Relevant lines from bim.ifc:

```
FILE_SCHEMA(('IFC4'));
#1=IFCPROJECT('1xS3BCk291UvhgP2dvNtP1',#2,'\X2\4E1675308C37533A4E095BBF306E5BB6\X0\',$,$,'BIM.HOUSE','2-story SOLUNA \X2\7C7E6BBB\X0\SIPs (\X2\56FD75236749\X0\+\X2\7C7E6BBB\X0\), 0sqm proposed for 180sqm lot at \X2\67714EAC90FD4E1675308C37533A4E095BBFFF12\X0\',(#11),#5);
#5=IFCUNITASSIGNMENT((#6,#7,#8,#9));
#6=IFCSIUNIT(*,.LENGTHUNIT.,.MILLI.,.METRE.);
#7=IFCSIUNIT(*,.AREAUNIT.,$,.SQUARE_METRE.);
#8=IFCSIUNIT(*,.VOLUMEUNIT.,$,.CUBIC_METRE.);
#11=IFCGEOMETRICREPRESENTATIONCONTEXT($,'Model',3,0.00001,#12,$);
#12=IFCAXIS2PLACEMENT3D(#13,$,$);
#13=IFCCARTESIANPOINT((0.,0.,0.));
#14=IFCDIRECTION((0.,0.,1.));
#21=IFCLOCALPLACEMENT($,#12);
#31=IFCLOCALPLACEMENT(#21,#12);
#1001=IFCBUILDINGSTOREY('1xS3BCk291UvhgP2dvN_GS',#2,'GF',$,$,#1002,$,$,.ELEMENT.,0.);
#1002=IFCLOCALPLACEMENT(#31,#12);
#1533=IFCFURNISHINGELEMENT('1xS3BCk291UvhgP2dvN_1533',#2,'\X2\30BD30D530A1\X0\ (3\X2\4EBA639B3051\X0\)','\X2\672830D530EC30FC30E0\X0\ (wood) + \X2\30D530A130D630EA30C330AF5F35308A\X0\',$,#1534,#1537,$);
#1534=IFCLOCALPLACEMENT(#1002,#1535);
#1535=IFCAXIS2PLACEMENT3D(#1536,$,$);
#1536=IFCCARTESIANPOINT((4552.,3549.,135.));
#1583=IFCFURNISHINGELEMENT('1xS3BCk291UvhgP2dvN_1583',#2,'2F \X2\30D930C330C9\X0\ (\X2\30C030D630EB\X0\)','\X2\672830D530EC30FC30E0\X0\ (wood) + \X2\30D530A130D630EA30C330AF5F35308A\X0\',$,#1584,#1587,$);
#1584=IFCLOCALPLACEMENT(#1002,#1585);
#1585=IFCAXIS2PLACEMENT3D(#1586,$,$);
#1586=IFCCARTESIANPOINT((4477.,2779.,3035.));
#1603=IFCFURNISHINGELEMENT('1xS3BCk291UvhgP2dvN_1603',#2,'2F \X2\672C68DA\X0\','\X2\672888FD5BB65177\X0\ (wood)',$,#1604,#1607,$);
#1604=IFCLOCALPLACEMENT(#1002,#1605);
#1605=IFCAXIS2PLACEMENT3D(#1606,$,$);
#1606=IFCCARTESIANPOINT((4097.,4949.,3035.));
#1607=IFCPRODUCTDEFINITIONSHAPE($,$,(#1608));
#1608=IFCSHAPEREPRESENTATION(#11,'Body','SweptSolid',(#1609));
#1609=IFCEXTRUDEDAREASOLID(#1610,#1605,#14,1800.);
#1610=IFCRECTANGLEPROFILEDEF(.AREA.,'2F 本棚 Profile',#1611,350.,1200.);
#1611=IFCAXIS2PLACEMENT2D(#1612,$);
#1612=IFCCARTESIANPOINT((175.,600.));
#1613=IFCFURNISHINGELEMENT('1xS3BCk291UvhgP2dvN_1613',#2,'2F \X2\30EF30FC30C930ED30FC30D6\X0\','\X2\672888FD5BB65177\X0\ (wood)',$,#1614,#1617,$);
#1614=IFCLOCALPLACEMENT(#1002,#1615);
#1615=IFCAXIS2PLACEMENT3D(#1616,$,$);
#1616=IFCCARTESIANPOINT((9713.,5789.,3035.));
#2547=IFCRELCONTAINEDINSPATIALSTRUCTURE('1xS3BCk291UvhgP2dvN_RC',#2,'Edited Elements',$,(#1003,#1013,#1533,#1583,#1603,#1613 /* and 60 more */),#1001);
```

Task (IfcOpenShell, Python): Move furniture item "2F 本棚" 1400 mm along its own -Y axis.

```python
import ifcopenshell
import ifcopenshell.api.geometry
import ifcopenshell.util.placement
import ifcopenshell.util.unit

model = ifcopenshell.open("bim.ifc")
unit_scale = ifcopenshell.util.unit.calculate_unit_scale(model)

item = model.by_guid("1xS3BCk291UvhgP2dvN_1603")
matrix = ifcopenshell.util.placement.get_local_placement(item.ObjectPlacement)
matrix[:3, 3] -= matrix[:3, 1] * 1.4 / unit_scale
ifcopenshell.api.geometry.edit_object_placement(model, product=item, matrix=matrix, is_si=False)

print(ifcopenshell.util.placement.get_local_placement(item.ObjectPlacement).round(3) + 0.0)

model.write("bim_v2.ifc")
```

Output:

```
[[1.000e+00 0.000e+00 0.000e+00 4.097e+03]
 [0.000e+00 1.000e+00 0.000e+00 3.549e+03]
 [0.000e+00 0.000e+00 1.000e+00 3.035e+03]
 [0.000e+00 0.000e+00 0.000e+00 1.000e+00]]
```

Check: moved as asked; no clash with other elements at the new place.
